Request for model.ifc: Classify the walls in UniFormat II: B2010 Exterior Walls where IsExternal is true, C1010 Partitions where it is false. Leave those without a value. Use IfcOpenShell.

First a look at what the model holds.

```python
import ifcopenshell
import ifcopenshell.util.element

model = ifcopenshell.open("model.ifc")
print(model.schema)
print("classifications:", [c.Name for c in model.by_type("IfcClassification")])
values = [ifcopenshell.util.element.get_pset(e, "Pset_WallCommon", "IsExternal") for e in model.by_type("IfcWall")]
for value in (True, False, None):
    print("IsExternal", value, values.count(value))
```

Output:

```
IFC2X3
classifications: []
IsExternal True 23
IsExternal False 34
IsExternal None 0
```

```python
import ifcopenshell
import ifcopenshell.api.classification
import ifcopenshell.util.element

model = ifcopenshell.open("model.ifc")

# IFC2X3 requires Source and Edition and has no link from the project to the system.
system = model.create_entity("IfcClassification", Source="ASTM", Edition="E1557", Name="UniFormat II")

walls = model.by_type("IfcWall")
external = {e: ifcopenshell.util.element.get_pset(e, "Pset_WallCommon", "IsExternal") for e in walls}
for flag, code, name in ((True, "B2010", "Exterior Walls"), (False, "C1010", "Partitions")):
    products = [e for e in walls if external[e] is flag]
    ifcopenshell.api.classification.add_reference(
        model, products=products, classification=system, identification=code, name=name
    )
    print(code, len(products))

model.write("model_updated.ifc")
```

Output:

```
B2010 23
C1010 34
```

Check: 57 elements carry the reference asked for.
